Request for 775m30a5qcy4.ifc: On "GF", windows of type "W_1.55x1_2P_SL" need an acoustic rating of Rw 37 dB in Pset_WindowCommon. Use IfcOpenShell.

First a look at what the model holds.

```python
import ifcopenshell
import ifcopenshell.util.element

model = ifcopenshell.open("775m30a5qcy4.ifc")
print(model.schema)
storey = next(s for s in model.by_type("IfcBuildingStorey") if s.Name == "GF")
windows = [e for e in ifcopenshell.util.element.get_decomposition(storey) if e.is_a("IfcWindow")]
seen = {}
for e in windows:
    element_type = ifcopenshell.util.element.get_type(e)
    key = (element_type.Name if element_type != e and element_type else None, ifcopenshell.util.element.get_pset(e, "Pset_WindowCommon", "AcousticRating"))
    seen[key] = seen.get(key, 0) + 1
for (name, value), count in sorted(seen.items(), key=str):
    print(count, "x", name, "|", value)
```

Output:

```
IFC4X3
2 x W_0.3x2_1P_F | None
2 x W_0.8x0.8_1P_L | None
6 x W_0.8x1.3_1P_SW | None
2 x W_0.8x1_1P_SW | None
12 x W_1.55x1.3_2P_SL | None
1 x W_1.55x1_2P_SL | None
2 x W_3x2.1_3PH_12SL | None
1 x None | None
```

```python
import ifcopenshell
import ifcopenshell.api.pset
import ifcopenshell.util.element

model = ifcopenshell.open("775m30a5qcy4.ifc")

storey = next(s for s in model.by_type("IfcBuildingStorey") if s.Name == "GF")
windows = [e for e in ifcopenshell.util.element.get_decomposition(storey) if e.is_a("IfcWindow")]

count = 0
for e in windows:
    element_type = ifcopenshell.util.element.get_type(e)
    if element_type in (None, e) or element_type.Name != "W_1.55x1_2P_SL":
        continue
    # add_pset returns the element's existing set when there is one.
    pset = ifcopenshell.api.pset.add_pset(model, product=e, name="Pset_WindowCommon")
    ifcopenshell.api.pset.edit_pset(model, pset=pset, properties={"AcousticRating": "Rw 37 dB"})
    count += 1

print(count, "windows updated")

model.write("775m30a5qcy4_updated.ifc")
```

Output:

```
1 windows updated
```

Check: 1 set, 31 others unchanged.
